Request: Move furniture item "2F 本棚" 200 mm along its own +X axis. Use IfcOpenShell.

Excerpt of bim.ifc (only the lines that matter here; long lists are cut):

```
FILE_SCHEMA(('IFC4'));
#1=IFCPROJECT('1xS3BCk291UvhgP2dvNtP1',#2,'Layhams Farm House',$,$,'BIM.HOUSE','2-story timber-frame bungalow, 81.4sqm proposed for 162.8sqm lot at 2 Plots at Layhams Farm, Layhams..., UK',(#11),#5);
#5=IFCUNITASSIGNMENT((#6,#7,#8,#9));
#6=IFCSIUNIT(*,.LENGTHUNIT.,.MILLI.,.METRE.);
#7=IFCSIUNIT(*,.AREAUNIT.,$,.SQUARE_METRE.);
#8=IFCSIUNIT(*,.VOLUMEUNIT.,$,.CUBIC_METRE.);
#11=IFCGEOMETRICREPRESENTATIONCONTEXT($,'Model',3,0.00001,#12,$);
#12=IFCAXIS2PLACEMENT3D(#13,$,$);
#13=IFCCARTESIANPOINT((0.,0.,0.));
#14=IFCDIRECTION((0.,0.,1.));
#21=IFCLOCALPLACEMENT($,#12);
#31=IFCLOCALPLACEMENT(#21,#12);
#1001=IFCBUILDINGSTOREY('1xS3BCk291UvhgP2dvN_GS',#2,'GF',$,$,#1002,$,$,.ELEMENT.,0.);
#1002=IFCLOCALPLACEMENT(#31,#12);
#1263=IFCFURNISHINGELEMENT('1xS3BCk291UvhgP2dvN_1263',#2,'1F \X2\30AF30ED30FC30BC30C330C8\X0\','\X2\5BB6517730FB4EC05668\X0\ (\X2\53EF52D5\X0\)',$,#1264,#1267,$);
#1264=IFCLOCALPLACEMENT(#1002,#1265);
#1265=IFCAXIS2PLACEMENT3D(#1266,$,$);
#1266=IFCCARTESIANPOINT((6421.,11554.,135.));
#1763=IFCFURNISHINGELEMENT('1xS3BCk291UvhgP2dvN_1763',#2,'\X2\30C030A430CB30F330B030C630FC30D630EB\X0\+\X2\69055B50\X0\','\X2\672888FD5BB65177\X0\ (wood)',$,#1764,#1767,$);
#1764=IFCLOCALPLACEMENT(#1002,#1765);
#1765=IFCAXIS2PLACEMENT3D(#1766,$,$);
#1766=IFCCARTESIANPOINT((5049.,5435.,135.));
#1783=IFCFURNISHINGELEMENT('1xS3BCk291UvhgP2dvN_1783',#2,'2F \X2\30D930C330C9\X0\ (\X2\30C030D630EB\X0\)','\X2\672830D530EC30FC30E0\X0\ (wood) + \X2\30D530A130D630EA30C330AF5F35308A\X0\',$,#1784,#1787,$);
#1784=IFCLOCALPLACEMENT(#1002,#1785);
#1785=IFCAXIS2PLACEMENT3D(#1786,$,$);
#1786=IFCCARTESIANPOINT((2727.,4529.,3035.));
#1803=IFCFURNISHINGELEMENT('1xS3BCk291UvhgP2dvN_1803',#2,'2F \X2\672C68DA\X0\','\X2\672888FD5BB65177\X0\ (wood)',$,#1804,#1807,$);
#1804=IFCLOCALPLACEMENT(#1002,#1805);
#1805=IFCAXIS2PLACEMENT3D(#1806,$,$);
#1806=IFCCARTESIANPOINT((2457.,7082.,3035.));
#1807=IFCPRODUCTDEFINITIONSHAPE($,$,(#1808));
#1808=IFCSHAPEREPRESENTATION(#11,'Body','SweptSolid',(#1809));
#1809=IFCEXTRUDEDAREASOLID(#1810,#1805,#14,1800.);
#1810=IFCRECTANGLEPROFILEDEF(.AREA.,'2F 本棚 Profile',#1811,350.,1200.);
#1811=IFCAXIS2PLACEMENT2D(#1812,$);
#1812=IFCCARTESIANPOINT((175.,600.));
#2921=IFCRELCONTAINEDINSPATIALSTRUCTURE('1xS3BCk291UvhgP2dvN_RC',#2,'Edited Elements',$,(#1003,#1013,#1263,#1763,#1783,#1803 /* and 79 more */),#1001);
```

```python
import ifcopenshell
import ifcopenshell.api.geometry
import ifcopenshell.util.placement
import ifcopenshell.util.unit

model = ifcopenshell.open("bim.ifc")
unit_scale = ifcopenshell.util.unit.calculate_unit_scale(model)

item = model.by_id(1803)
matrix = ifcopenshell.util.placement.get_local_placement(item.ObjectPlacement)
matrix[:3, 3] += matrix[:3, 0] * 0.2 / unit_scale
ifcopenshell.api.geometry.edit_object_placement(model, product=item, matrix=matrix, is_si=False)

print(ifcopenshell.util.placement.get_local_placement(item.ObjectPlacement).round(3) + 0.0)

model.write("bim_rev.ifc")
```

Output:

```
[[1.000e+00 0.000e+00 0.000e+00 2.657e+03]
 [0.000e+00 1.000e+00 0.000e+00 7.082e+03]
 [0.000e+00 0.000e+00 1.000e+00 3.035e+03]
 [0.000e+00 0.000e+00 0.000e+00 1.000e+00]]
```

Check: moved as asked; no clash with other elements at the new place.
